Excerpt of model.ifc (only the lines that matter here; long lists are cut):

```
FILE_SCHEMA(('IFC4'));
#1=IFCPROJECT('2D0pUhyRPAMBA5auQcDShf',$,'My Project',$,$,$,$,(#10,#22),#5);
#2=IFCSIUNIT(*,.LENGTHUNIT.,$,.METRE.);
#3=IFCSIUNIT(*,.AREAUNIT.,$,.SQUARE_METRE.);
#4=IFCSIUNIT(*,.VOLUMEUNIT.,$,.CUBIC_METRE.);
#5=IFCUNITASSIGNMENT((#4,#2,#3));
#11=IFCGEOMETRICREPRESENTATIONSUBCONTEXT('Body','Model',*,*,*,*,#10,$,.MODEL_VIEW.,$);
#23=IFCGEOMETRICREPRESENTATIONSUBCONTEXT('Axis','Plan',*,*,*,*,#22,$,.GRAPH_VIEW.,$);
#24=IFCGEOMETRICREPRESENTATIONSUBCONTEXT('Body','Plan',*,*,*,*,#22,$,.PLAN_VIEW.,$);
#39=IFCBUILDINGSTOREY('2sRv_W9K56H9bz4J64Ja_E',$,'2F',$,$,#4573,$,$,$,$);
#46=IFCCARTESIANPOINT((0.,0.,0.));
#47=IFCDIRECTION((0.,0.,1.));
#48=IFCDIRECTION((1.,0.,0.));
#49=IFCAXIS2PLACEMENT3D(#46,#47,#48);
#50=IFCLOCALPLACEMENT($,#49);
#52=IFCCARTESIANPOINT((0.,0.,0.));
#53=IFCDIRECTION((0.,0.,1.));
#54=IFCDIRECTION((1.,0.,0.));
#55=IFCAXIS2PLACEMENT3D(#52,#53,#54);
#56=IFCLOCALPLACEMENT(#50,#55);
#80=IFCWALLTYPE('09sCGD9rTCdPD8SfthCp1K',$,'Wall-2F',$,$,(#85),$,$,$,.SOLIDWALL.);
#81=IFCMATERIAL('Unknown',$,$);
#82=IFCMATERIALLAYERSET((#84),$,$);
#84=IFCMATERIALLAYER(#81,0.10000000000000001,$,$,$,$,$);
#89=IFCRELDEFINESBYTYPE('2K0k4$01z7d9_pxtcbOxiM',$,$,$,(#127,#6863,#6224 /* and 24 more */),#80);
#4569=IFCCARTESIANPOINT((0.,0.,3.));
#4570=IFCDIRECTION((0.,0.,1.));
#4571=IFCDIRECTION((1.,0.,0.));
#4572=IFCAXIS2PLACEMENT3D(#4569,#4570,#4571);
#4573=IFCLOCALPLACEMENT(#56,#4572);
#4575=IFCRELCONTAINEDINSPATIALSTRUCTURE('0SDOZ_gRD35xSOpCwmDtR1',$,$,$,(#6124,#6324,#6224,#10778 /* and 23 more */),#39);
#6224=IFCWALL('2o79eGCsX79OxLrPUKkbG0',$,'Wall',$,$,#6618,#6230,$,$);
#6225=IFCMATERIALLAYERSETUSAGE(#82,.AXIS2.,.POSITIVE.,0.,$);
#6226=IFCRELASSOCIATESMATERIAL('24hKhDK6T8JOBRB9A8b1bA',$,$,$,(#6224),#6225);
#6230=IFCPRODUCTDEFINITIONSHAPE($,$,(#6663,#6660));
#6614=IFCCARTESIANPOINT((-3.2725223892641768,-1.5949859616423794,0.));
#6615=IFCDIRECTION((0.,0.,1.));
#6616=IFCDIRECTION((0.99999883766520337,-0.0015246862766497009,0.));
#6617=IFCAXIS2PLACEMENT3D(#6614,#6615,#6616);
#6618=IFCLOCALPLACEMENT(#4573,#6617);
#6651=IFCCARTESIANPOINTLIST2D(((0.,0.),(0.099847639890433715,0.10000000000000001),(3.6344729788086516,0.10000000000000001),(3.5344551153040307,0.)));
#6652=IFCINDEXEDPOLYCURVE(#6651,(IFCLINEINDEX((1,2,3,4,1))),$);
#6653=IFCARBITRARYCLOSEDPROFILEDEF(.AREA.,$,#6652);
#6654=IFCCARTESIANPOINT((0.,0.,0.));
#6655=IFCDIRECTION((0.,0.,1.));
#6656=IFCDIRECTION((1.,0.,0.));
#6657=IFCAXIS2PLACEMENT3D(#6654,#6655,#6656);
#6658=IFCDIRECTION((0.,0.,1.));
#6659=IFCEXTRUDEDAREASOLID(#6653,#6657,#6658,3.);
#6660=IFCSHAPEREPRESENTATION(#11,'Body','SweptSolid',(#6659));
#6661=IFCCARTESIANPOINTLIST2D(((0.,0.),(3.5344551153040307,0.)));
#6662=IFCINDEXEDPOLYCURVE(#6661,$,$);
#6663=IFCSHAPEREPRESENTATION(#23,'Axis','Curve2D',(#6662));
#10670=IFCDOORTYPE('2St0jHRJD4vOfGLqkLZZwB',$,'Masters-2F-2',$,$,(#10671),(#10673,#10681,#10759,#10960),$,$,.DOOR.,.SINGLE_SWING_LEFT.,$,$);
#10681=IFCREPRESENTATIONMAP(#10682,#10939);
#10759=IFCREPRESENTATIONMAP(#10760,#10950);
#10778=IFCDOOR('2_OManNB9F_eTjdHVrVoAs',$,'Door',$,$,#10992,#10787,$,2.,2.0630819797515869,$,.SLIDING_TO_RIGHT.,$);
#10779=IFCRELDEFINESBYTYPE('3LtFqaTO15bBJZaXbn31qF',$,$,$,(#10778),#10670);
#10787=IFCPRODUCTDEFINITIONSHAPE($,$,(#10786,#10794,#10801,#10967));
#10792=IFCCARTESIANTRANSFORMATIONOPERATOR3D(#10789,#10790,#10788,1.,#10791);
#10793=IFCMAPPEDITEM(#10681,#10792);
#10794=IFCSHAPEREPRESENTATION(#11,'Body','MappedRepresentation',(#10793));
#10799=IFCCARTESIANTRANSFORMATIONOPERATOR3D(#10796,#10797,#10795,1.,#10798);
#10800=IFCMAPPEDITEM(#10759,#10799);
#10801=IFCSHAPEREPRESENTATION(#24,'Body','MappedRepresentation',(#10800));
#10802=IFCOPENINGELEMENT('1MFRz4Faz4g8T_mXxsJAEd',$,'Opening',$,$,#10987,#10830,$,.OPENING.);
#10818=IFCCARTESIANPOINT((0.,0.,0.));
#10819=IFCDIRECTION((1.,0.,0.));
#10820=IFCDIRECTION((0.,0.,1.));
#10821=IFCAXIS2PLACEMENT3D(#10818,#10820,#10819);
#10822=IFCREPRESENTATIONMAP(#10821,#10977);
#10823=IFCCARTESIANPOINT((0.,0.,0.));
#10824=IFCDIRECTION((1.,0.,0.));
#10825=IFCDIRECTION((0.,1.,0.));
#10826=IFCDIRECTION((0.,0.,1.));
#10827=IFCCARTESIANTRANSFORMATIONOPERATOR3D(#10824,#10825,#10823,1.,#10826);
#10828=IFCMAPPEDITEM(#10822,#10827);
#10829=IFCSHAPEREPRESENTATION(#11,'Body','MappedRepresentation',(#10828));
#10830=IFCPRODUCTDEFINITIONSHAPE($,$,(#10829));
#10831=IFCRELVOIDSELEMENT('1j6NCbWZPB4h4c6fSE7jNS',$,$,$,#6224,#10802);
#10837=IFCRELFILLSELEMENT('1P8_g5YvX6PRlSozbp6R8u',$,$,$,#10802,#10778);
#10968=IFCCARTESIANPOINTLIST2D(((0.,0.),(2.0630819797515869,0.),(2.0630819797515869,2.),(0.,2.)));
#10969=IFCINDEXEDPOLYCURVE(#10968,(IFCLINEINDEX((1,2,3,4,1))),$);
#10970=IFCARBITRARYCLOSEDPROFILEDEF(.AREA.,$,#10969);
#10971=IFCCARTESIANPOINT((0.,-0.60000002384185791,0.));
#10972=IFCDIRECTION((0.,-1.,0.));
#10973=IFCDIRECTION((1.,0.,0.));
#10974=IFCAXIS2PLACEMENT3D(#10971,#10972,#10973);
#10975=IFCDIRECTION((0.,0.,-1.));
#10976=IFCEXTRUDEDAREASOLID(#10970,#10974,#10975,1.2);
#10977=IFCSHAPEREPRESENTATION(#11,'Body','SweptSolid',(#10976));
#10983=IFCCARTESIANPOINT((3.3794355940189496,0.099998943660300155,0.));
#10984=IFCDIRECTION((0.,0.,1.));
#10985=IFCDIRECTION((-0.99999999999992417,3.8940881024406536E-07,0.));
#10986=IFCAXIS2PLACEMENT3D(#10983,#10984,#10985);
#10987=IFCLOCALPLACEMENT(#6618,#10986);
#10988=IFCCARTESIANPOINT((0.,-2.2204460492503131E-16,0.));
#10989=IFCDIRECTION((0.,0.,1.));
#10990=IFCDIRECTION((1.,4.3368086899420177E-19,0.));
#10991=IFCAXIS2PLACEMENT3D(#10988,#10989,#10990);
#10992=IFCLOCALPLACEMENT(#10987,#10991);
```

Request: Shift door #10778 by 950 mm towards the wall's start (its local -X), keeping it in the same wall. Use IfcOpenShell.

```python
import ifcopenshell
import ifcopenshell.api.geometry
import ifcopenshell.util.placement

model = ifcopenshell.open("model.ifc")

door = model.by_id(10778)
opening = door.FillsVoids[0].RelatingOpeningElement
wall = opening.VoidsElements[0].RelatingBuildingElement

wall_matrix = ifcopenshell.util.placement.get_local_placement(wall.ObjectPlacement)
shift = wall_matrix[:3, 0] * -0.95
before = ifcopenshell.util.placement.get_local_placement(door.ObjectPlacement)[:3, 3].copy()

# The door is placed relative to its opening, so it follows when the opening moves.
matrix = ifcopenshell.util.placement.get_local_placement(opening.ObjectPlacement)
matrix[:3, 3] += shift
ifcopenshell.api.geometry.edit_object_placement(
    model, product=opening, matrix=matrix, is_si=False, should_transform_children=True
)

after = ifcopenshell.util.placement.get_local_placement(door.ObjectPlacement)[:3, 3]
print("door moved by", (after - before).round(3) + 0.0)

model.write("model_v2.ifc")
```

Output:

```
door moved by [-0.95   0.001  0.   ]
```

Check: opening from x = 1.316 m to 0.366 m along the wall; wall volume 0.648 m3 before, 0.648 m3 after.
